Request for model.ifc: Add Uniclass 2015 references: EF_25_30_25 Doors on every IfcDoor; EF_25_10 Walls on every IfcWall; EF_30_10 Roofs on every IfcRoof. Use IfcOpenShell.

First a look at what the model holds.

```python
import ifcopenshell

model = ifcopenshell.open("model.ifc")
print(model.schema)
print("classifications:", [c.Name for c in model.by_type("IfcClassification")])
for ifc_class in ("IfcDoor", "IfcRoof", "IfcStair", "IfcWall", "IfcWindow"):
    print(ifc_class, len(model.by_type(ifc_class)))
```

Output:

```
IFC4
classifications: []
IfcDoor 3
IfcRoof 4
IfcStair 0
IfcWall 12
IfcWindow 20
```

```python
import ifcopenshell
import ifcopenshell.api.classification

model = ifcopenshell.open("model.ifc")

system = ifcopenshell.api.classification.add_classification(model, classification="Uniclass 2015")

codes = {
    "IfcDoor": ("EF_25_30_25", "Doors"),
    "IfcWall": ("EF_25_10", "Walls"),
    "IfcRoof": ("EF_30_10", "Roofs"),
}
for ifc_class, (code, name) in codes.items():
    products = model.by_type(ifc_class)
    ifcopenshell.api.classification.add_reference(
        model, products=products, classification=system, identification=code, name=name
    )
    print(code, len(products))

model.write("model_edited.ifc")
```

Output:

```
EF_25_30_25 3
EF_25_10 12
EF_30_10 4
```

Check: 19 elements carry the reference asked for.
